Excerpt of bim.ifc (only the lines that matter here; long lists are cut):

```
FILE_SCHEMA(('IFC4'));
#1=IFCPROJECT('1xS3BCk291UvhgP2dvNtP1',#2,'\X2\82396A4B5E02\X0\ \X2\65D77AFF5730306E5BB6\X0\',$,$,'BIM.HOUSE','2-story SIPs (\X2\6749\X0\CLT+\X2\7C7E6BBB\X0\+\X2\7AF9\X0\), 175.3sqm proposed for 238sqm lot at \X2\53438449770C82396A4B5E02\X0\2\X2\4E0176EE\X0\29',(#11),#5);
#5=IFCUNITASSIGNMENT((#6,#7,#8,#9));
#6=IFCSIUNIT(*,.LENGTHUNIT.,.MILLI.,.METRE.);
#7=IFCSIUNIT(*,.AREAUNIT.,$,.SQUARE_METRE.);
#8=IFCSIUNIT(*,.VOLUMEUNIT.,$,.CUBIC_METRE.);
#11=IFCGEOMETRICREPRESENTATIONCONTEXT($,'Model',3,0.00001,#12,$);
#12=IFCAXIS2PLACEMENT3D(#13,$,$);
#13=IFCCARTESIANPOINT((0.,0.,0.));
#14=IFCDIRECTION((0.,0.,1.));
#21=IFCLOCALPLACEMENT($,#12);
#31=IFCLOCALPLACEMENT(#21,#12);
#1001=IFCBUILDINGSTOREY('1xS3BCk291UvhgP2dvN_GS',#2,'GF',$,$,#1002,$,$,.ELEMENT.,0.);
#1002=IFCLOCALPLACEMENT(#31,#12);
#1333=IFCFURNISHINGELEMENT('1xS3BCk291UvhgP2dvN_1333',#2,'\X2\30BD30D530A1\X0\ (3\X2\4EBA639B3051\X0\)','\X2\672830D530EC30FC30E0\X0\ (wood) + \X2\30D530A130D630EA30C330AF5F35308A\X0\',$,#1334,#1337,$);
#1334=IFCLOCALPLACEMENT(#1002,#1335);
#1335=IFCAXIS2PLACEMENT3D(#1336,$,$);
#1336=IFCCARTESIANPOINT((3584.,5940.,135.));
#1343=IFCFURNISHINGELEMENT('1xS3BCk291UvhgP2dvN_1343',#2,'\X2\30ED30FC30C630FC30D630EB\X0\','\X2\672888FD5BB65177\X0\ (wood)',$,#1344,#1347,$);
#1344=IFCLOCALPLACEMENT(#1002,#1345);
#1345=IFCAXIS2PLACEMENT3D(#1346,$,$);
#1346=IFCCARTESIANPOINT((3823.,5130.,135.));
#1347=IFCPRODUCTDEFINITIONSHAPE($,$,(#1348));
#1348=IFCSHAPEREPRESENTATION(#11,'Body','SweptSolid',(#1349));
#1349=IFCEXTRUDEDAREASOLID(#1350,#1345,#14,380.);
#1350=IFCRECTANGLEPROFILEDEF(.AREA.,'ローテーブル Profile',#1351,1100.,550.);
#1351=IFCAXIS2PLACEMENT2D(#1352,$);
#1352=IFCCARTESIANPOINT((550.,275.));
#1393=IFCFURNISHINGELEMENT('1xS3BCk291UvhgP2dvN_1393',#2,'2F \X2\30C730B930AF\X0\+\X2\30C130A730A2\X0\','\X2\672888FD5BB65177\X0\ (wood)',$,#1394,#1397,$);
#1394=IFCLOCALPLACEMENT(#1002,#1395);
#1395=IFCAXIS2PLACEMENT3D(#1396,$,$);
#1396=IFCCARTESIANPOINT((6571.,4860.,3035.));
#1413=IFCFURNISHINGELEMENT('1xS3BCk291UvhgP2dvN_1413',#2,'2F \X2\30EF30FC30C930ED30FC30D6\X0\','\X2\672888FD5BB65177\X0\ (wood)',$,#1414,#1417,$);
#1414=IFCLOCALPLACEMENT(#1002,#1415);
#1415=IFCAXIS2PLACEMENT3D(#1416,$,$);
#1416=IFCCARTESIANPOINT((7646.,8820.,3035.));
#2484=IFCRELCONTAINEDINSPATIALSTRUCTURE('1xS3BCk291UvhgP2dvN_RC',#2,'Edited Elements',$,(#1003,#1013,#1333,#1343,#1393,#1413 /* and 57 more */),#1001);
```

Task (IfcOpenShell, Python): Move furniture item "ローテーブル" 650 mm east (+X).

```python
import ifcopenshell
import ifcopenshell.api.geometry
import ifcopenshell.util.placement
import ifcopenshell.util.unit

model = ifcopenshell.open("bim.ifc")
unit_scale = ifcopenshell.util.unit.calculate_unit_scale(model)

item = model.by_id(1343)
matrix = ifcopenshell.util.placement.get_local_placement(item.ObjectPlacement)
matrix[0, 3] += 0.65 / unit_scale
ifcopenshell.api.geometry.edit_object_placement(model, product=item, matrix=matrix, is_si=False)

print(ifcopenshell.util.placement.get_local_placement(item.ObjectPlacement).round(3) + 0.0)

model.write("bim_updated.ifc")
```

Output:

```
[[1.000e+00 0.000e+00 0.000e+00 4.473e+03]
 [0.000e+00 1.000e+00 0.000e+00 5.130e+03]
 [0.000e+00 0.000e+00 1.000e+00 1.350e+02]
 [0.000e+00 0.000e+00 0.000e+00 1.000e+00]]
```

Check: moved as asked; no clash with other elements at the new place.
